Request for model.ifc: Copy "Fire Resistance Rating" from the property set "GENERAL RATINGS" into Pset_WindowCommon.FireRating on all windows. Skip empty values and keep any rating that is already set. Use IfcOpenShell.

First a look at what the model holds.

```python
import ifcopenshell
import ifcopenshell.util.element

model = ifcopenshell.open("model.ifc")
print(model.schema)
windows = model.by_type("IfcWindow")
print(len(windows), "windows")
for e in windows[:8]:
    source = ifcopenshell.util.element.get_pset(e, "GENERAL RATINGS", "Fire Resistance Rating")
    target = ifcopenshell.util.element.get_pset(e, "Pset_WindowCommon", "FireRating")
    print(e.id(), repr(source), repr(target), sep=" | ")
```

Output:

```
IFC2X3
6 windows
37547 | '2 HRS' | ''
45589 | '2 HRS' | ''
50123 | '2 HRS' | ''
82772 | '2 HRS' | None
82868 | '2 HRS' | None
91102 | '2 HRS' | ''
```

```python
import ifcopenshell
import ifcopenshell.api.pset
import ifcopenshell.util.element

model = ifcopenshell.open("model.ifc")

count = 0
for e in model.by_type("IfcWindow"):
    value = ifcopenshell.util.element.get_pset(e, "GENERAL RATINGS", "Fire Resistance Rating")
    current = ifcopenshell.util.element.get_pset(e, "Pset_WindowCommon", "FireRating")
    if not value or not value.strip() or current:
        continue
    # add_pset returns the element's existing set when there is one.
    pset = ifcopenshell.api.pset.add_pset(model, product=e, name="Pset_WindowCommon")
    ifcopenshell.api.pset.edit_pset(model, pset=pset, properties={"FireRating": value})
    count += 1

print(count, "windows updated")

model.write("model-out.ifc")
```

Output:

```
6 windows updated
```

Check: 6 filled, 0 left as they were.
